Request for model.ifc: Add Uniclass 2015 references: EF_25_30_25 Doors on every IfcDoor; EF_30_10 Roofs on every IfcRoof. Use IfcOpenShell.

First a look at what the model holds.

```python
import ifcopenshell

model = ifcopenshell.open("model.ifc")
print(model.schema)
print("classifications:", [c.Name for c in model.by_type("IfcClassification")])
for ifc_class in ("IfcDoor", "IfcRoof", "IfcStair", "IfcWall", "IfcWindow"):
    print(ifc_class, len(model.by_type(ifc_class)))
```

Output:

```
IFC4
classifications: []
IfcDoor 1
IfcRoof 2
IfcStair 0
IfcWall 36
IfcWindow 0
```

```python
import ifcopenshell
import ifcopenshell.api.classification

model = ifcopenshell.open("model.ifc")

system = ifcopenshell.api.classification.add_classification(model, classification="Uniclass 2015")

codes = {
    "IfcDoor": ("EF_25_30_25", "Doors"),
    "IfcRoof": ("EF_30_10", "Roofs"),
}
for ifc_class, (code, name) in codes.items():
    products = model.by_type(ifc_class)
    ifcopenshell.api.classification.add_reference(
        model, products=products, classification=system, identification=code, name=name
    )
    print(code, len(products))

model.write("model_updated.ifc")
```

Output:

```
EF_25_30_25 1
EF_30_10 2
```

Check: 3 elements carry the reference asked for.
